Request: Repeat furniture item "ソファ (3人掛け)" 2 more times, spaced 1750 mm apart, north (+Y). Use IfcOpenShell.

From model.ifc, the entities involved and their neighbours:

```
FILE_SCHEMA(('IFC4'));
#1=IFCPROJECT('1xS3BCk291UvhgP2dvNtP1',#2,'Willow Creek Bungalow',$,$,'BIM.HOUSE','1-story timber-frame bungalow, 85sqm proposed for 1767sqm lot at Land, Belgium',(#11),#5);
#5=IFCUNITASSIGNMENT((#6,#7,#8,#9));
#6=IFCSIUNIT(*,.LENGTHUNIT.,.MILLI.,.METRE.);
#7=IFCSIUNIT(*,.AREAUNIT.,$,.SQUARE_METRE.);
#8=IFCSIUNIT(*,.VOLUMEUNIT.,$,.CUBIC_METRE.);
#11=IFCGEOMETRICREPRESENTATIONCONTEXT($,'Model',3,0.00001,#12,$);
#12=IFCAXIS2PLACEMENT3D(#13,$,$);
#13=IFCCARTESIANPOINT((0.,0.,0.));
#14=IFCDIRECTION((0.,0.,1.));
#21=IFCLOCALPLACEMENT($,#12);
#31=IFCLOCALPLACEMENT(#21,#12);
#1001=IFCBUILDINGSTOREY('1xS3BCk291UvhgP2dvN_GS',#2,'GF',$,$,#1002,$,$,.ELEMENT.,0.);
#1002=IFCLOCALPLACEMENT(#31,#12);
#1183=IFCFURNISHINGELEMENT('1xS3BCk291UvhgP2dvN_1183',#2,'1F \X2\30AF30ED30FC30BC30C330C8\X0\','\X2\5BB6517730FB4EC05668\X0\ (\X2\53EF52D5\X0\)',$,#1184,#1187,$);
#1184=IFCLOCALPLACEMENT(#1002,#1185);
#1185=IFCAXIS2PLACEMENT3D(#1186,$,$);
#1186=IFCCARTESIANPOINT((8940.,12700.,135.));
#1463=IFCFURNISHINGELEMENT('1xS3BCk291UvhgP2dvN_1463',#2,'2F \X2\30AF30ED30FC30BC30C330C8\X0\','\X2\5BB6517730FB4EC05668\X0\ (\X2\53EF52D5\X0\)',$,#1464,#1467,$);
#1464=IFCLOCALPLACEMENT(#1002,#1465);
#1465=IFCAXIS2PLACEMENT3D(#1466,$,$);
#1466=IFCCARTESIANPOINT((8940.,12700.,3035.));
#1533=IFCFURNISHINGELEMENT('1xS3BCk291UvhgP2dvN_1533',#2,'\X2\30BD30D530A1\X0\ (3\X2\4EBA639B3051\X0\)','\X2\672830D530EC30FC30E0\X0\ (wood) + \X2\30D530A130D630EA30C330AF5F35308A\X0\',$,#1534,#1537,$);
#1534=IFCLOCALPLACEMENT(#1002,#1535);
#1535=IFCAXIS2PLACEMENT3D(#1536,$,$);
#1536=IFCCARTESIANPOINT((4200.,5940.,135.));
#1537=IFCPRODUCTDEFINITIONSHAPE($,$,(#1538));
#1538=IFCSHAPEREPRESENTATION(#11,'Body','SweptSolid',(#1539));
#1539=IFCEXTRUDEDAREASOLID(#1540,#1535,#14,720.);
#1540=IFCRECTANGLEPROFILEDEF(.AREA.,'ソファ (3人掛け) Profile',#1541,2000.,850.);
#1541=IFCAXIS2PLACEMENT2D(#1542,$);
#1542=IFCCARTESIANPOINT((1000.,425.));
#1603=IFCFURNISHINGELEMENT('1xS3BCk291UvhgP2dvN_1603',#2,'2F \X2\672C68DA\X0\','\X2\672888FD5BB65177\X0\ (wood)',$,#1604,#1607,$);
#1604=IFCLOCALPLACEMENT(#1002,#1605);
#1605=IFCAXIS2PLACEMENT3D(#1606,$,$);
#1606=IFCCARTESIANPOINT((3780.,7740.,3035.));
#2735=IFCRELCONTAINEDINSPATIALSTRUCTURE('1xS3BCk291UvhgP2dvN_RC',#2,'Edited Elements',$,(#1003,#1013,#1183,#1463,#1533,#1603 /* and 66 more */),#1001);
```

```python
import numpy as np
import ifcopenshell
import ifcopenshell.api.geometry
import ifcopenshell.api.root
import ifcopenshell.util.element
import ifcopenshell.util.placement
import ifcopenshell.util.unit

model = ifcopenshell.open("model.ifc")
unit_scale = ifcopenshell.util.unit.calculate_unit_scale(model)


def reuse_history(source, copy):
    """copy_class also copies each property set's owner history, people and application; keep the originals."""
    for rel in copy.IsDefinedBy:
        if rel.is_a("IfcRelDefinesByProperties") and (history := rel.RelatingPropertyDefinition.OwnerHistory):
            rel.RelatingPropertyDefinition.OwnerHistory = source.OwnerHistory
            ifcopenshell.util.element.remove_deep2(model, history)


source = model.by_guid("1xS3BCk291UvhgP2dvN_1533")
base = ifcopenshell.util.placement.get_local_placement(source.ObjectPlacement)
step = np.array([0.0, 1.0, 0.0]) * 1.75 / unit_scale

for i in range(1, 3):
    copy = ifcopenshell.api.root.copy_class(model, product=source)
    copy.Representation = ifcopenshell.util.element.copy_deep(
        model, source.Representation, exclude=["IfcGeometricRepresentationContext", "IfcRepresentationMap"]
    )
    reuse_history(source, copy)
    matrix = base.copy()
    matrix[:3, 3] += i * step
    print("added at", matrix[:3, 3].round(3) + 0.0)
    ifcopenshell.api.geometry.edit_object_placement(model, product=copy, matrix=matrix, is_si=False)

model.write("model_updated.ifc")
```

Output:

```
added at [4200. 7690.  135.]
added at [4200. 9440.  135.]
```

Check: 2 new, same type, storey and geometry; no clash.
